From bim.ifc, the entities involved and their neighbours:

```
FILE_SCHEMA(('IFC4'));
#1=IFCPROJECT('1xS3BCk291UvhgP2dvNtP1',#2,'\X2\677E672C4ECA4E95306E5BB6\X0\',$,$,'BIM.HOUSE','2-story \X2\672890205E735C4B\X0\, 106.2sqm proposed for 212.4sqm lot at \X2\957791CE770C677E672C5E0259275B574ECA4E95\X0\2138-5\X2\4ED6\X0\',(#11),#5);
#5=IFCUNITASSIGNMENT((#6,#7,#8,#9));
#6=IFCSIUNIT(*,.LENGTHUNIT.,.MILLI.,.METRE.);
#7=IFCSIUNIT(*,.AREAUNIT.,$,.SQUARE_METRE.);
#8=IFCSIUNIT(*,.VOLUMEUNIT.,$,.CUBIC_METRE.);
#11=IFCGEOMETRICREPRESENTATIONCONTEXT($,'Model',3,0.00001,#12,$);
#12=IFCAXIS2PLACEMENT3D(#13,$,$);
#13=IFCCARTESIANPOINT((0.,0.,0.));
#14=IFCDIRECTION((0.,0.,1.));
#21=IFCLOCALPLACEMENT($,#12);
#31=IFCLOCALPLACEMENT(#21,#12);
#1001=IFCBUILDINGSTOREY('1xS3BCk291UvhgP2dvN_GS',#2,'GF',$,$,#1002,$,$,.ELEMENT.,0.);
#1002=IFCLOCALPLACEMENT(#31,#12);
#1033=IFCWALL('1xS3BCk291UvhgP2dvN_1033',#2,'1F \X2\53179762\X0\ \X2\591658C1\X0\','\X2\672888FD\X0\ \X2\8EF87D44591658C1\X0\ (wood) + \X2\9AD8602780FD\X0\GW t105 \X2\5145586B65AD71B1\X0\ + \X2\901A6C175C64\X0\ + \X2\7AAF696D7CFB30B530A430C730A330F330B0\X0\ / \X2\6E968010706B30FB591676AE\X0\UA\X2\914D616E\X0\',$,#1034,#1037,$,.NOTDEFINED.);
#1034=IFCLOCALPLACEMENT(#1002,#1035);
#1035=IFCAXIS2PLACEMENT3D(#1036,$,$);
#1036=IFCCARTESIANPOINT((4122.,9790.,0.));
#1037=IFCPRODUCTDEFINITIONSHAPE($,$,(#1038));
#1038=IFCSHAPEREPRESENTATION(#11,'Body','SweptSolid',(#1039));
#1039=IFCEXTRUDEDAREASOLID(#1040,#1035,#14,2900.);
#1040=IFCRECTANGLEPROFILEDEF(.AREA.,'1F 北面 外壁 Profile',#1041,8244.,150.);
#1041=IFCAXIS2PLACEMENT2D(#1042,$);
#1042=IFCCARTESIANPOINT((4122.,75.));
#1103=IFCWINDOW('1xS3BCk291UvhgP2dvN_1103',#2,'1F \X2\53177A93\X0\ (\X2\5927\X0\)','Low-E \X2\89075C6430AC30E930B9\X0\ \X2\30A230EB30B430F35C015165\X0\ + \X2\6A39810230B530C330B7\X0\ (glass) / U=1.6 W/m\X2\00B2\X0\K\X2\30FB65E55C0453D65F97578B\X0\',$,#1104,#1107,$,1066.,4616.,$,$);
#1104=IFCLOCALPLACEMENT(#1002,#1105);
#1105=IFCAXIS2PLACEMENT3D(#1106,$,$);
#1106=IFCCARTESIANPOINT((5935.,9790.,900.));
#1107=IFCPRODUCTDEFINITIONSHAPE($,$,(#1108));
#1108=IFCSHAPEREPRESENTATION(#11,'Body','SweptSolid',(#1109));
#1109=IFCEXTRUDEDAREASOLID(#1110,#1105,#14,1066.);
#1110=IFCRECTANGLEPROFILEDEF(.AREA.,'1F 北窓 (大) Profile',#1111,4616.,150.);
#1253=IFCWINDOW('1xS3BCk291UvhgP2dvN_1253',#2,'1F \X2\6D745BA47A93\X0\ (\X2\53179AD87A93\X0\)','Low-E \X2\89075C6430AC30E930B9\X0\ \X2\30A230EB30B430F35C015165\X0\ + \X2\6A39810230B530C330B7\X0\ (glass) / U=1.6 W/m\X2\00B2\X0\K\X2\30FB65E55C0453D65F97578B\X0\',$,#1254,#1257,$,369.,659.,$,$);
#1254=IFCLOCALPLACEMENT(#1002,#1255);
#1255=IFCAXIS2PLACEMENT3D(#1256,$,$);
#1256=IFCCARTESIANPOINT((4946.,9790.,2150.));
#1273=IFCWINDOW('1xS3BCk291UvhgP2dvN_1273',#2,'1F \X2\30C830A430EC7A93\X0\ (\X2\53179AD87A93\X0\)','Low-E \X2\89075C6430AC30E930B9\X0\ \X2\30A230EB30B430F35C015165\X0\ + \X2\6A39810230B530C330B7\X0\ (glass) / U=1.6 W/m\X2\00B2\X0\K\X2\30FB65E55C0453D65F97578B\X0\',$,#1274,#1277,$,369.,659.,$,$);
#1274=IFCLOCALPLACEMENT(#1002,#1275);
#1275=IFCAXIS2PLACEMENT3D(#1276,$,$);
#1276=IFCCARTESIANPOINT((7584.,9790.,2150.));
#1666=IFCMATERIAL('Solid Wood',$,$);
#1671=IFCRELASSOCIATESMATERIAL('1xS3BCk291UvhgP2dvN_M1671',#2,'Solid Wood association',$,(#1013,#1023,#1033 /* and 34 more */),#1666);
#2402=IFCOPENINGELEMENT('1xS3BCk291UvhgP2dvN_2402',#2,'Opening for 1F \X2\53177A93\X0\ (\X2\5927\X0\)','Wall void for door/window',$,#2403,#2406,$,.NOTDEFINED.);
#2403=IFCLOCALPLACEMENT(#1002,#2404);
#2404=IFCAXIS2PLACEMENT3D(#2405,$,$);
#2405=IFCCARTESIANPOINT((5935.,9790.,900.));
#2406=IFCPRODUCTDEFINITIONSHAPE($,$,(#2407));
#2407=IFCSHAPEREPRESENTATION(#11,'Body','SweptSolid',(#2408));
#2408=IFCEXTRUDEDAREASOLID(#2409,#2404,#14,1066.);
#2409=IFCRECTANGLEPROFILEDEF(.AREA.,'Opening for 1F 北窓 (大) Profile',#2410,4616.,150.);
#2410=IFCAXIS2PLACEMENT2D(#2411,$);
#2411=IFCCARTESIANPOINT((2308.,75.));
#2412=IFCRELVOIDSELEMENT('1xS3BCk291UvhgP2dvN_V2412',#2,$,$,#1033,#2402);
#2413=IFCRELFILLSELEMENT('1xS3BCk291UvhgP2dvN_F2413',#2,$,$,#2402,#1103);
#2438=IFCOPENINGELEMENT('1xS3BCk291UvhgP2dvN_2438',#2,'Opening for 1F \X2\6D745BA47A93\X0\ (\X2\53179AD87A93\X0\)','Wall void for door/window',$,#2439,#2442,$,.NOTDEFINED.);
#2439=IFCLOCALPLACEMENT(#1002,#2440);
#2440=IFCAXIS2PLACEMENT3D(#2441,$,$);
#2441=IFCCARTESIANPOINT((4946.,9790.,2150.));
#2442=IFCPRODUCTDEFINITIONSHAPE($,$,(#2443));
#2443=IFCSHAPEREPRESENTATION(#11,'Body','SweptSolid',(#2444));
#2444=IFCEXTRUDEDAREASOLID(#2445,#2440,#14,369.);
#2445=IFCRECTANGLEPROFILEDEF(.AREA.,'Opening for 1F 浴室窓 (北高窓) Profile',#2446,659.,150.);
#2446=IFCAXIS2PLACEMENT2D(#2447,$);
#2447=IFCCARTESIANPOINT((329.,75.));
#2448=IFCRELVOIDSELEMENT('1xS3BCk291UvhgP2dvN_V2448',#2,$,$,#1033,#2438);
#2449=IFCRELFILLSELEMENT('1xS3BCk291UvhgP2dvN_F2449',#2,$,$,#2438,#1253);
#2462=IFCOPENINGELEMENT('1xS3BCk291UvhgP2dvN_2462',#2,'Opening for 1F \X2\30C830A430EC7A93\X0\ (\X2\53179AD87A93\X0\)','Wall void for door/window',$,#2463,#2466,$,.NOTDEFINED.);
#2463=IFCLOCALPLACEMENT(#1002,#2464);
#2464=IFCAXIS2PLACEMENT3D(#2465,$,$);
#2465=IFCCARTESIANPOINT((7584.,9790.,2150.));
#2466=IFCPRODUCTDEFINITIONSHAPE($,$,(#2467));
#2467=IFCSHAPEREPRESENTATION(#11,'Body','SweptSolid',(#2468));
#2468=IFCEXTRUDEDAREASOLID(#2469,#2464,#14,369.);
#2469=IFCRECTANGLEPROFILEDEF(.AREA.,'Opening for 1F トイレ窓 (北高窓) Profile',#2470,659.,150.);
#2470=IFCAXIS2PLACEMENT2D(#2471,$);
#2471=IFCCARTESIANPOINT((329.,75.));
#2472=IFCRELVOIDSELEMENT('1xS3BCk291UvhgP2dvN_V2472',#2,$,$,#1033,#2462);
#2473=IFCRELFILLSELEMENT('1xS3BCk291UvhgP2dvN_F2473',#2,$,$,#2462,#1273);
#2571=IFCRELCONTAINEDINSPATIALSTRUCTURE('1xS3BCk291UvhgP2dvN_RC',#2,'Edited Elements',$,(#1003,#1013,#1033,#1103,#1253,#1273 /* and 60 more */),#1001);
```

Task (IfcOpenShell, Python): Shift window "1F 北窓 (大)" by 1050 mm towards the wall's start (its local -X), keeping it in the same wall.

```python
import ifcopenshell
import ifcopenshell.api.geometry
import ifcopenshell.util.placement
import ifcopenshell.util.unit

model = ifcopenshell.open("bim.ifc")
unit_scale = ifcopenshell.util.unit.calculate_unit_scale(model)

window = model.by_id(1103)
opening = window.FillsVoids[0].RelatingOpeningElement
wall = opening.VoidsElements[0].RelatingBuildingElement

wall_matrix = ifcopenshell.util.placement.get_local_placement(wall.ObjectPlacement)
shift = wall_matrix[:3, 0] * -1.05 / unit_scale
before = ifcopenshell.util.placement.get_local_placement(window.ObjectPlacement)[:3, 3].copy()

# The window is not placed relative to its opening, so move both.
for product in (opening, window):
    matrix = ifcopenshell.util.placement.get_local_placement(product.ObjectPlacement)
    matrix[:3, 3] += shift
    ifcopenshell.api.geometry.edit_object_placement(model, product=product, matrix=matrix, is_si=False)

after = ifcopenshell.util.placement.get_local_placement(window.ObjectPlacement)[:3, 3]
print("window moved by", (after - before).round(3) + 0.0)

model.write("bim_v2.ifc")
```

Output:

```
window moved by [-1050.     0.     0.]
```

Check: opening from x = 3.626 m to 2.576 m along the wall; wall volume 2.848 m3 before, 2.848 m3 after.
